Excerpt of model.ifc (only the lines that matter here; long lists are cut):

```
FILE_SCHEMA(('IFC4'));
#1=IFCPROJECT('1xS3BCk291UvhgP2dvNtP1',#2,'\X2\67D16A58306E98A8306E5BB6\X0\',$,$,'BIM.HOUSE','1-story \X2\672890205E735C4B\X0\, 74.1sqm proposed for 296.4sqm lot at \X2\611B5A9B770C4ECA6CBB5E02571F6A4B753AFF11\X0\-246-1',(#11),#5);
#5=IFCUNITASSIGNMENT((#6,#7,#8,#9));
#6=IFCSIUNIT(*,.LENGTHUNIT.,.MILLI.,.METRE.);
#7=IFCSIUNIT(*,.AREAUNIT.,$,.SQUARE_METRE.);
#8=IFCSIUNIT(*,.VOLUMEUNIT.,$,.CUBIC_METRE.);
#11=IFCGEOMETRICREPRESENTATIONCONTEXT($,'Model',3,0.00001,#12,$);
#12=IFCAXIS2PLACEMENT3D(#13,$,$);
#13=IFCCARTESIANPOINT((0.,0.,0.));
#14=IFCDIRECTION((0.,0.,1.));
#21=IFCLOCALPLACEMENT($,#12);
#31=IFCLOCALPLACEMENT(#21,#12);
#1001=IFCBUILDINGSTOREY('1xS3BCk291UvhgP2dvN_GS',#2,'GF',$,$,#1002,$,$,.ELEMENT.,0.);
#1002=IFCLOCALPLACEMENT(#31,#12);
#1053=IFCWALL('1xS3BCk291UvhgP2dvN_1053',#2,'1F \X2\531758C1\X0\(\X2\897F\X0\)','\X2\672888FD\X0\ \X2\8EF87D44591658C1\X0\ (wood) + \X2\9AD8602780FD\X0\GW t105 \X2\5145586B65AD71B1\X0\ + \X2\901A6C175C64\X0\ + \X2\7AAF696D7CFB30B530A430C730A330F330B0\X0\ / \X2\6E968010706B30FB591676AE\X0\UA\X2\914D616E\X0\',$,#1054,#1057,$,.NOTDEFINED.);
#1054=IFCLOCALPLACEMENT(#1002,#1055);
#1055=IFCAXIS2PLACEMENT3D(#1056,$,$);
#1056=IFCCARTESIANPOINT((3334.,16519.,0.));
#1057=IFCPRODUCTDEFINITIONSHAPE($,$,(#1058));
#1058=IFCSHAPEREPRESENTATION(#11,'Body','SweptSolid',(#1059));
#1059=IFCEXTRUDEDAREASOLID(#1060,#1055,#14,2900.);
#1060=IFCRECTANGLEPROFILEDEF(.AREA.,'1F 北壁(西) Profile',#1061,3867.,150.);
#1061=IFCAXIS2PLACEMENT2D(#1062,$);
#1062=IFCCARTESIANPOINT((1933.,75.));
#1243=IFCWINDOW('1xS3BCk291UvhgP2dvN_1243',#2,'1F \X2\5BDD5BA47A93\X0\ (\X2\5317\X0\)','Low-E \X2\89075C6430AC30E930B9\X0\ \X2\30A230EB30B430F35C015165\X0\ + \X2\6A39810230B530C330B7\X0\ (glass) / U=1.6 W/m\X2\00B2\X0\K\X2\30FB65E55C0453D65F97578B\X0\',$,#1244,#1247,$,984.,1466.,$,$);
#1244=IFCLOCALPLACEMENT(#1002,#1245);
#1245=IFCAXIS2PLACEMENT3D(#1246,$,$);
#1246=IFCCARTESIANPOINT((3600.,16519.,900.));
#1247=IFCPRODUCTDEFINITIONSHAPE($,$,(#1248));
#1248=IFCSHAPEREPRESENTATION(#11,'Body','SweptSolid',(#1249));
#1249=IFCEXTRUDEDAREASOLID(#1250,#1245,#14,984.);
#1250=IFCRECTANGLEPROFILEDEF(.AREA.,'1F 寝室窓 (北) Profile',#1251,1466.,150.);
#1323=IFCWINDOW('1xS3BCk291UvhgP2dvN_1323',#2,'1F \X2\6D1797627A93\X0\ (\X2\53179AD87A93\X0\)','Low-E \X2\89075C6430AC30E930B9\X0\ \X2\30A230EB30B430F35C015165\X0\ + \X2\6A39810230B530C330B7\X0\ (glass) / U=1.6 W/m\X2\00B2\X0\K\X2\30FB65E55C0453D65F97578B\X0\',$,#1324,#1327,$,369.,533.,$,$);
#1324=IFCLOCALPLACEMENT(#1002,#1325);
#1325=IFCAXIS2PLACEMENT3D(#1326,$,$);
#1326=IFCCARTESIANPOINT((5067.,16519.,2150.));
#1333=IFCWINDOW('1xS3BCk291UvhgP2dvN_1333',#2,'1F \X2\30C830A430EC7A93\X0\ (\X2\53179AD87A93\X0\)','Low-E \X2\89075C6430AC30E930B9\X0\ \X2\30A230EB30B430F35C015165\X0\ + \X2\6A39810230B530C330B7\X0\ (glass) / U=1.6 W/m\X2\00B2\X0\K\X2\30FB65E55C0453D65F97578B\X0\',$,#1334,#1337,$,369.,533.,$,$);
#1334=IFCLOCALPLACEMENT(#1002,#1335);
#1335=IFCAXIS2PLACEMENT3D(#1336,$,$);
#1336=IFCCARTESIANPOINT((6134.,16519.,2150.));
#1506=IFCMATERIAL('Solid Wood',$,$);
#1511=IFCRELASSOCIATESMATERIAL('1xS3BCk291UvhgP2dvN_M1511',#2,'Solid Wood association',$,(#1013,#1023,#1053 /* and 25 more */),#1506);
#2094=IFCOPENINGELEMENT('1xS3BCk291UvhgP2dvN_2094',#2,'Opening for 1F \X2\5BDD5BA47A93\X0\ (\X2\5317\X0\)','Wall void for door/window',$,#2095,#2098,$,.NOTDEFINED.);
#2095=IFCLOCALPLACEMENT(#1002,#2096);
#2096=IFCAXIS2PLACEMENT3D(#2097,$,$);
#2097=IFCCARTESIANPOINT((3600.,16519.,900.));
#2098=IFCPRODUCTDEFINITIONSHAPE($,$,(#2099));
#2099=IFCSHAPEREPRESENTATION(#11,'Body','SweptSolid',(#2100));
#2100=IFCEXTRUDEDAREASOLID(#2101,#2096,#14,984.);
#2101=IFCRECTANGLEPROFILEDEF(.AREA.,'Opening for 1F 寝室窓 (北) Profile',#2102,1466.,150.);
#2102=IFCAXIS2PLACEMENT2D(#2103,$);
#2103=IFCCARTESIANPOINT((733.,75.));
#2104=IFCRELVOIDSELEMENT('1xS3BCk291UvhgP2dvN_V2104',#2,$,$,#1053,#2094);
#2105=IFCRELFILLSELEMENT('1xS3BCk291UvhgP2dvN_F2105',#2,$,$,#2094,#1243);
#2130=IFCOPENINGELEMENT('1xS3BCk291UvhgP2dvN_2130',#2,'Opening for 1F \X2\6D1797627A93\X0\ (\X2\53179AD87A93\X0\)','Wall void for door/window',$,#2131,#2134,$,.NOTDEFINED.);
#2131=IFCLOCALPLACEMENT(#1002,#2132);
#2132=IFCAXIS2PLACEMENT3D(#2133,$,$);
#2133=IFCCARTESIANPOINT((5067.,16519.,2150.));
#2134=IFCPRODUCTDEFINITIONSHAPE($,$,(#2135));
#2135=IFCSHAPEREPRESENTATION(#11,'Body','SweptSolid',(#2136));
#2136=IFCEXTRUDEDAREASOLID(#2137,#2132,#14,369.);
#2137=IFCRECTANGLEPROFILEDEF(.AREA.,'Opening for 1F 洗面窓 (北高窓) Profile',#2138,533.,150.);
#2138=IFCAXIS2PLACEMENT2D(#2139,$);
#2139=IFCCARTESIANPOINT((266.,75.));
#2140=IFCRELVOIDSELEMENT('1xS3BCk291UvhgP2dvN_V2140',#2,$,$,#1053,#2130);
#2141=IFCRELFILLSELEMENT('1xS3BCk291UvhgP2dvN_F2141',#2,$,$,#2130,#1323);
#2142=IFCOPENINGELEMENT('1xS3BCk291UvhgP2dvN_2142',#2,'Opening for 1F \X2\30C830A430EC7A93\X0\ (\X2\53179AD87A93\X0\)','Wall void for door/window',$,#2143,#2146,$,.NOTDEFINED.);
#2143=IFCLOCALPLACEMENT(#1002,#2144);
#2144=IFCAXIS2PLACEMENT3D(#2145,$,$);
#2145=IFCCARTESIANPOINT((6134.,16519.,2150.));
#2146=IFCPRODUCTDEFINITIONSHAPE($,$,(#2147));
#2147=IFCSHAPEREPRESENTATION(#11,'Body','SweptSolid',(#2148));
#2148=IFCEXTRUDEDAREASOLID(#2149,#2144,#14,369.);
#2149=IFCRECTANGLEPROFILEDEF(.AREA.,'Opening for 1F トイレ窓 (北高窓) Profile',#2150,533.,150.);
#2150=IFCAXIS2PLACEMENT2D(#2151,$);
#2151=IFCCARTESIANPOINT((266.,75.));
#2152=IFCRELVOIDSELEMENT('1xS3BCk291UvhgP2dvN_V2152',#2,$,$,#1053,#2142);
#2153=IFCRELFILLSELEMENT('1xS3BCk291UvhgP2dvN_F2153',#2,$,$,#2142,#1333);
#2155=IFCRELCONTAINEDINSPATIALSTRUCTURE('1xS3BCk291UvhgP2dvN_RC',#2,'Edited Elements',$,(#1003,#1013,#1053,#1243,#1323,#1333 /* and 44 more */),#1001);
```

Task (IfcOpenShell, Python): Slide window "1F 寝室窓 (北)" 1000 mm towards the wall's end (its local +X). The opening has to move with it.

```python
import ifcopenshell
import ifcopenshell.api.geometry
import ifcopenshell.util.placement
import ifcopenshell.util.unit

model = ifcopenshell.open("model.ifc")
unit_scale = ifcopenshell.util.unit.calculate_unit_scale(model)

window = model.by_guid("1xS3BCk291UvhgP2dvN_1243")
opening = window.FillsVoids[0].RelatingOpeningElement
wall = opening.VoidsElements[0].RelatingBuildingElement

wall_matrix = ifcopenshell.util.placement.get_local_placement(wall.ObjectPlacement)
shift = wall_matrix[:3, 0] * 1 / unit_scale
before = ifcopenshell.util.placement.get_local_placement(window.ObjectPlacement)[:3, 3].copy()

# The window is not placed relative to its opening, so move both.
for product in (opening, window):
    matrix = ifcopenshell.util.placement.get_local_placement(product.ObjectPlacement)
    matrix[:3, 3] += shift
    ifcopenshell.api.geometry.edit_object_placement(model, product=product, matrix=matrix, is_si=False)

after = ifcopenshell.util.placement.get_local_placement(window.ObjectPlacement)[:3, 3]
print("window moved by", (after - before).round(3) + 0.0)

model.write("model_edited.ifc")
```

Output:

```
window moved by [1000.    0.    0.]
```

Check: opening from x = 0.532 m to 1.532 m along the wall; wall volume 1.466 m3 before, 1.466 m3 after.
